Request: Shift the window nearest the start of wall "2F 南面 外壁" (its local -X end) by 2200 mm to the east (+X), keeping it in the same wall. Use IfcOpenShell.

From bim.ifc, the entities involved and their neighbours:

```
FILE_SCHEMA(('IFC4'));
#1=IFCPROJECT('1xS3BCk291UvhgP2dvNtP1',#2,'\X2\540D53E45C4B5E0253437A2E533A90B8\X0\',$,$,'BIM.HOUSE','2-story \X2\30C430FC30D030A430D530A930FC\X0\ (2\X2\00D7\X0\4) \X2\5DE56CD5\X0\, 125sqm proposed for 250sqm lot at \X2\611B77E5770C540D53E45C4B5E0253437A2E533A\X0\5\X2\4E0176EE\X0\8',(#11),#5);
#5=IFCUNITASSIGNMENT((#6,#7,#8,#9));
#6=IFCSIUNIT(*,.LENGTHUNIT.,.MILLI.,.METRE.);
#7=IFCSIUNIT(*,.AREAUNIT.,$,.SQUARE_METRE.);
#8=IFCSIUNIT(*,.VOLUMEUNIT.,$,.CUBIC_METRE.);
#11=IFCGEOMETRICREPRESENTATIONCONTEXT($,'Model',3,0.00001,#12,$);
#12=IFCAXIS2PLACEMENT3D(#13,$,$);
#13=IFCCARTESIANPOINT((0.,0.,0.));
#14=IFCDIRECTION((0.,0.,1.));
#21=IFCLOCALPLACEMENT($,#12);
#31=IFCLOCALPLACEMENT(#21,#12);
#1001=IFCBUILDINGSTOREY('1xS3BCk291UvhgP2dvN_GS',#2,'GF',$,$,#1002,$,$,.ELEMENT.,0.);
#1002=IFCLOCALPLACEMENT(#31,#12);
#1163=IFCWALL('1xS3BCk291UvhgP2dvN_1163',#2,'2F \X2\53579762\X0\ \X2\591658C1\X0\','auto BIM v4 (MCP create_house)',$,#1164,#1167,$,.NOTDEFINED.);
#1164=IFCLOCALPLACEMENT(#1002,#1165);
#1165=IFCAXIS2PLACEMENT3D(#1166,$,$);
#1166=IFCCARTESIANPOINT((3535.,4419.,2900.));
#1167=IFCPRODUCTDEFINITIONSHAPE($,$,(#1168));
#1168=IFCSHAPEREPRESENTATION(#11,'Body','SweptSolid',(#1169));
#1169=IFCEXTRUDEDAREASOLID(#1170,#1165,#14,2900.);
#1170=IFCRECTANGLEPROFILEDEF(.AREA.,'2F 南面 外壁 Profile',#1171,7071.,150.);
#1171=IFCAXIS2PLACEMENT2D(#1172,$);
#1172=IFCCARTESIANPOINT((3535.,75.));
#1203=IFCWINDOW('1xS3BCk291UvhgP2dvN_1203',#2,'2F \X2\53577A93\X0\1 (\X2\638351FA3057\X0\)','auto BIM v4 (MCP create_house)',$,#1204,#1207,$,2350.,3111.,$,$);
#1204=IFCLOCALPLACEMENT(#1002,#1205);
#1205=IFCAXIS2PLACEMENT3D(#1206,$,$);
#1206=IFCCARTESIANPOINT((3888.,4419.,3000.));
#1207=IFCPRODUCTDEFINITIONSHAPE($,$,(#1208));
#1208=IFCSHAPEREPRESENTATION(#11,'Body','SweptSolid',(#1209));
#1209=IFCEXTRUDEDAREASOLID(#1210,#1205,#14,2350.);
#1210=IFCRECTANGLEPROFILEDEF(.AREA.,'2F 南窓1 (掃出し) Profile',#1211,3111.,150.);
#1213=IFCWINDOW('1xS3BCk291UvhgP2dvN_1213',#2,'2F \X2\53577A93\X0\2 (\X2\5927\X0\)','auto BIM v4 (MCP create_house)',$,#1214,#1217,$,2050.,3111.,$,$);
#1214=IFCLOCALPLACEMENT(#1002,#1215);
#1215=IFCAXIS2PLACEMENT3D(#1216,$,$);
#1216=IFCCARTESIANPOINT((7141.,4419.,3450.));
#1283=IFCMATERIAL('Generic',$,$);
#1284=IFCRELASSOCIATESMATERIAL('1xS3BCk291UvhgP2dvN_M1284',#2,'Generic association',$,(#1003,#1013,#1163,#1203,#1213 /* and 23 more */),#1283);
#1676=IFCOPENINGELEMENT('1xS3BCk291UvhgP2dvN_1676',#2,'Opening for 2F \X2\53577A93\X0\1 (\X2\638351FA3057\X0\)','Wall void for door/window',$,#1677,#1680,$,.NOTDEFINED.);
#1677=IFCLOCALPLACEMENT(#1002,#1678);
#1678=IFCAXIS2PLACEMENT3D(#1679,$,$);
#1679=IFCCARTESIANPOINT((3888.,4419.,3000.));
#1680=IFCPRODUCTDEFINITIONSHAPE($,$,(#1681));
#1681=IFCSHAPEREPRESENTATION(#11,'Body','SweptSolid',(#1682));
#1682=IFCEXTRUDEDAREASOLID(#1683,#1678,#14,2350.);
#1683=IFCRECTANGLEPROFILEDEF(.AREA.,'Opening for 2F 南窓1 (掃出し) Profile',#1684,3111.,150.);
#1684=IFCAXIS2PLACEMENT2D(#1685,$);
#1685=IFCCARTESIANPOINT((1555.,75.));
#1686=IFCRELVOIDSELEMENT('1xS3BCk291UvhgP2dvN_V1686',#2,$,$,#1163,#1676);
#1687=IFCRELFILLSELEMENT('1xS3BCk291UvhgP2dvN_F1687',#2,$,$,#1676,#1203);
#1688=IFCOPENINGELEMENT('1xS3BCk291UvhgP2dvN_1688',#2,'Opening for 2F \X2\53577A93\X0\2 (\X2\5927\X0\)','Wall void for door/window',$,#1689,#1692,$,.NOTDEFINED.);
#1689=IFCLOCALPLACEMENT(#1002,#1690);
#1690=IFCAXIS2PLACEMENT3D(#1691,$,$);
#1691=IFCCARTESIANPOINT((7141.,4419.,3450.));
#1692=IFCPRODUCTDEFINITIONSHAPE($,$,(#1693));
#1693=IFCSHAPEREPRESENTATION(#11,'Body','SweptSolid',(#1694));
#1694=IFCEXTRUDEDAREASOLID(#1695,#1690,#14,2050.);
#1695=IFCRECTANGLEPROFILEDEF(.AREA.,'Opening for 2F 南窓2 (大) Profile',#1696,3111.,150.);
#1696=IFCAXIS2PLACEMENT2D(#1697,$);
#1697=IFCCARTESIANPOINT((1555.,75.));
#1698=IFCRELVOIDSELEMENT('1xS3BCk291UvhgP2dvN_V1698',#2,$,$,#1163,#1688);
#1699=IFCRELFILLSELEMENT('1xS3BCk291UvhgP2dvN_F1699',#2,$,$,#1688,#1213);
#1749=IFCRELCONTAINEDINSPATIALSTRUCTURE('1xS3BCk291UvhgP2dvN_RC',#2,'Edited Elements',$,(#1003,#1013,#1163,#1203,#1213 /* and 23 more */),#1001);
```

```python
import ifcopenshell
import ifcopenshell.api.geometry
import ifcopenshell.util.placement
import ifcopenshell.util.unit

model = ifcopenshell.open("bim.ifc")
unit_scale = ifcopenshell.util.unit.calculate_unit_scale(model)

window = model.by_id(1203)
opening = window.FillsVoids[0].RelatingOpeningElement
wall = opening.VoidsElements[0].RelatingBuildingElement

wall_matrix = ifcopenshell.util.placement.get_local_placement(wall.ObjectPlacement)
shift = wall_matrix[:3, 0] * 2.2 / unit_scale
before = ifcopenshell.util.placement.get_local_placement(window.ObjectPlacement)[:3, 3].copy()

# The window is not placed relative to its opening, so move both.
for product in (opening, window):
    matrix = ifcopenshell.util.placement.get_local_placement(product.ObjectPlacement)
    matrix[:3, 3] += shift
    ifcopenshell.api.geometry.edit_object_placement(model, product=product, matrix=matrix, is_si=False)

after = ifcopenshell.util.placement.get_local_placement(window.ObjectPlacement)[:3, 3]
print("window moved by", (after - before).round(3) + 0.0)

model.write("bim_v2.ifc")
```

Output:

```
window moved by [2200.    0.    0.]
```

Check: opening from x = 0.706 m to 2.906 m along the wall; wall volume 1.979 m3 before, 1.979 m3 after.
